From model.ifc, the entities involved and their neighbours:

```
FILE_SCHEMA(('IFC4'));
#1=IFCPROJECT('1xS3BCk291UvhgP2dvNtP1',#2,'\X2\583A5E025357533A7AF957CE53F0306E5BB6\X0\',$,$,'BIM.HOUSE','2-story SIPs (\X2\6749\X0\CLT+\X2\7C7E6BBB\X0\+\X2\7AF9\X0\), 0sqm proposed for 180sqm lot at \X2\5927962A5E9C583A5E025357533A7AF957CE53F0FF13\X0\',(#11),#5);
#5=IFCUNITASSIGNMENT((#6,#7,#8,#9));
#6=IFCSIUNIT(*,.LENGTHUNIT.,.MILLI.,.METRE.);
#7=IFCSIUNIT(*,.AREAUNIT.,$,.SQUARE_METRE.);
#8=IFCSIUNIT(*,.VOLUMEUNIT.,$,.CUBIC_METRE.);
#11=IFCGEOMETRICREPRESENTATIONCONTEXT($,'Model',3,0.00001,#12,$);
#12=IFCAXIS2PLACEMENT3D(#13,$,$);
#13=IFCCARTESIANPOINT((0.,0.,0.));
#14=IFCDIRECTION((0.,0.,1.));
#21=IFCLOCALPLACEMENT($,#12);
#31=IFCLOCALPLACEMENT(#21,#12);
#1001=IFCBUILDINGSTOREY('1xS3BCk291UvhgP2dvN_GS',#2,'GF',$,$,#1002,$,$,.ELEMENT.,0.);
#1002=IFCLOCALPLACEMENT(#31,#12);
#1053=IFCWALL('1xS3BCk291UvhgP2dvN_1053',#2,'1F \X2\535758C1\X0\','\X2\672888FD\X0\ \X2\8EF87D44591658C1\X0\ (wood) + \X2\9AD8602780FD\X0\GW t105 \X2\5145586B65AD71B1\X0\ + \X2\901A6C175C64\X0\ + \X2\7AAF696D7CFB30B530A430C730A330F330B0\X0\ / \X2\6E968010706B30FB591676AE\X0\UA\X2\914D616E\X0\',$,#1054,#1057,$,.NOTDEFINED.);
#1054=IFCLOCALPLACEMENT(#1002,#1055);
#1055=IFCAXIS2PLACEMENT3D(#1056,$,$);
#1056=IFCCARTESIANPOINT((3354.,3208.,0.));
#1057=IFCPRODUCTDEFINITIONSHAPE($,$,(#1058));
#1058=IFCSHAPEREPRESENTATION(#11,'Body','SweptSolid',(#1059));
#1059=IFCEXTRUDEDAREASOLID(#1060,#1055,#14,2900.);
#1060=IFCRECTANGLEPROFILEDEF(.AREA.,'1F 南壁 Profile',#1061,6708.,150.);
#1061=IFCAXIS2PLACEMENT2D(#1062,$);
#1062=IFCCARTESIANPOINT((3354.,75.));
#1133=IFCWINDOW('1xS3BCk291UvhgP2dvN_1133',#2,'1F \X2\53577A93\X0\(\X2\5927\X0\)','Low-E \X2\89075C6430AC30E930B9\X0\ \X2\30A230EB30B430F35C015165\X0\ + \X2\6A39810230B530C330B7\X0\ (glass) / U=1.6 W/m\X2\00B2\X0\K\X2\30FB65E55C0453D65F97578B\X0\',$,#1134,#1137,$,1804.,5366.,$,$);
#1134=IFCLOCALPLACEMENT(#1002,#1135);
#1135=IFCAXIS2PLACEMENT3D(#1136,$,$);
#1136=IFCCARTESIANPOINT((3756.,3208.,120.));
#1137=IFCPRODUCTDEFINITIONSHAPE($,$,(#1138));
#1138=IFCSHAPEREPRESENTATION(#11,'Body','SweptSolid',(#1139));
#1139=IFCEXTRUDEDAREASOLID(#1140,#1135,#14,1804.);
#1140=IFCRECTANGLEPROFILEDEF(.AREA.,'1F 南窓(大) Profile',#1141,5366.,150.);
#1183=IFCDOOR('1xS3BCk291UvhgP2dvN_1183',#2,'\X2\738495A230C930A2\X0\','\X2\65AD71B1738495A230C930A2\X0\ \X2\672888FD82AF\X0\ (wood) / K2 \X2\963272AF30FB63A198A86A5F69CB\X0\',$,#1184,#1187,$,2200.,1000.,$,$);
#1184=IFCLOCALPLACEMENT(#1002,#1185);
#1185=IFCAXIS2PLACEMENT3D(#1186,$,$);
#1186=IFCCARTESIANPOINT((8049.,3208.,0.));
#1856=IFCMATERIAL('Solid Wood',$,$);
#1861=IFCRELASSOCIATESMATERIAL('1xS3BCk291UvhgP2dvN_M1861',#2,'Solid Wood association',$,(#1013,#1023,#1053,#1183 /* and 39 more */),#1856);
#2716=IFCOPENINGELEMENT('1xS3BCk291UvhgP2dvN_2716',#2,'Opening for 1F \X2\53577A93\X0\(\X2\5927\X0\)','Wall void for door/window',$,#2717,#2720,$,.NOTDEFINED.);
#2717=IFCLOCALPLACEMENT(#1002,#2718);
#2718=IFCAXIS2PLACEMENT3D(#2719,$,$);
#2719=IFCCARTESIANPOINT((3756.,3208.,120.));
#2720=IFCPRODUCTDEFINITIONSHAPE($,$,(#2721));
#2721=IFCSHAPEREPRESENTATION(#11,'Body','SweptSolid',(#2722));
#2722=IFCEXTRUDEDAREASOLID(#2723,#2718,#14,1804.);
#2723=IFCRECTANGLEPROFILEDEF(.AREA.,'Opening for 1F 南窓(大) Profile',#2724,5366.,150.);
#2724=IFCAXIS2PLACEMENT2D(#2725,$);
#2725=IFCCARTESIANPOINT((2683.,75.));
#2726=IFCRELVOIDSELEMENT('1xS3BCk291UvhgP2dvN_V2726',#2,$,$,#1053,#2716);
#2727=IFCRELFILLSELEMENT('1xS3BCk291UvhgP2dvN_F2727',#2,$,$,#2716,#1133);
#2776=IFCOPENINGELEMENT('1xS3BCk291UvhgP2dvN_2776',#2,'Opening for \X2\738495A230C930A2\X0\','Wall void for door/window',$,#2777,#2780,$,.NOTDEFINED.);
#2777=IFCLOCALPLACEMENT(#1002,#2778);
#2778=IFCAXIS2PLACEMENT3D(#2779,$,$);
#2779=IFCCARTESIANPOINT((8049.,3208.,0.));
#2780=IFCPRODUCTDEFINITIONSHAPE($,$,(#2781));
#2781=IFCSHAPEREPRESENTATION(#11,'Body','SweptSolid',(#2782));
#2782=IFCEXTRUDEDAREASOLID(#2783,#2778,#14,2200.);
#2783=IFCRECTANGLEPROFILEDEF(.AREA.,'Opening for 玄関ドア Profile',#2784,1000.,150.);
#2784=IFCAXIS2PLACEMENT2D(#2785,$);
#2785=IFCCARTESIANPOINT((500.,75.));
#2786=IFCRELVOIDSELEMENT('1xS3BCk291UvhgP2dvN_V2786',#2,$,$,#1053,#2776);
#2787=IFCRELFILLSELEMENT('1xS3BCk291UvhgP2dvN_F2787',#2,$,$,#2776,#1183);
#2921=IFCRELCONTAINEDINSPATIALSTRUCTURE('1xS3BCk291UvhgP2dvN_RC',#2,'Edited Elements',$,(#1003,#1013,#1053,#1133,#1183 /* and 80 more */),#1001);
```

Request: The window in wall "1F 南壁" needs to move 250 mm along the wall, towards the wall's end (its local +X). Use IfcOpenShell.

```python
import ifcopenshell
import ifcopenshell.api.geometry
import ifcopenshell.util.placement
import ifcopenshell.util.unit

model = ifcopenshell.open("model.ifc")
unit_scale = ifcopenshell.util.unit.calculate_unit_scale(model)

window = model.by_guid("1xS3BCk291UvhgP2dvN_1133")
opening = window.FillsVoids[0].RelatingOpeningElement
wall = opening.VoidsElements[0].RelatingBuildingElement

wall_matrix = ifcopenshell.util.placement.get_local_placement(wall.ObjectPlacement)
shift = wall_matrix[:3, 0] * 0.25 / unit_scale
before = ifcopenshell.util.placement.get_local_placement(window.ObjectPlacement)[:3, 3].copy()

# The window is not placed relative to its opening, so move both.
for product in (opening, window):
    matrix = ifcopenshell.util.placement.get_local_placement(product.ObjectPlacement)
    matrix[:3, 3] += shift
    ifcopenshell.api.geometry.edit_object_placement(model, product=product, matrix=matrix, is_si=False)

after = ifcopenshell.util.placement.get_local_placement(window.ObjectPlacement)[:3, 3]
print("window moved by", (after - before).round(3) + 0.0)

model.write("model-out.ifc")
```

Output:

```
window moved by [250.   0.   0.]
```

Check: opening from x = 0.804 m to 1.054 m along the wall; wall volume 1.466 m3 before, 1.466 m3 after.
